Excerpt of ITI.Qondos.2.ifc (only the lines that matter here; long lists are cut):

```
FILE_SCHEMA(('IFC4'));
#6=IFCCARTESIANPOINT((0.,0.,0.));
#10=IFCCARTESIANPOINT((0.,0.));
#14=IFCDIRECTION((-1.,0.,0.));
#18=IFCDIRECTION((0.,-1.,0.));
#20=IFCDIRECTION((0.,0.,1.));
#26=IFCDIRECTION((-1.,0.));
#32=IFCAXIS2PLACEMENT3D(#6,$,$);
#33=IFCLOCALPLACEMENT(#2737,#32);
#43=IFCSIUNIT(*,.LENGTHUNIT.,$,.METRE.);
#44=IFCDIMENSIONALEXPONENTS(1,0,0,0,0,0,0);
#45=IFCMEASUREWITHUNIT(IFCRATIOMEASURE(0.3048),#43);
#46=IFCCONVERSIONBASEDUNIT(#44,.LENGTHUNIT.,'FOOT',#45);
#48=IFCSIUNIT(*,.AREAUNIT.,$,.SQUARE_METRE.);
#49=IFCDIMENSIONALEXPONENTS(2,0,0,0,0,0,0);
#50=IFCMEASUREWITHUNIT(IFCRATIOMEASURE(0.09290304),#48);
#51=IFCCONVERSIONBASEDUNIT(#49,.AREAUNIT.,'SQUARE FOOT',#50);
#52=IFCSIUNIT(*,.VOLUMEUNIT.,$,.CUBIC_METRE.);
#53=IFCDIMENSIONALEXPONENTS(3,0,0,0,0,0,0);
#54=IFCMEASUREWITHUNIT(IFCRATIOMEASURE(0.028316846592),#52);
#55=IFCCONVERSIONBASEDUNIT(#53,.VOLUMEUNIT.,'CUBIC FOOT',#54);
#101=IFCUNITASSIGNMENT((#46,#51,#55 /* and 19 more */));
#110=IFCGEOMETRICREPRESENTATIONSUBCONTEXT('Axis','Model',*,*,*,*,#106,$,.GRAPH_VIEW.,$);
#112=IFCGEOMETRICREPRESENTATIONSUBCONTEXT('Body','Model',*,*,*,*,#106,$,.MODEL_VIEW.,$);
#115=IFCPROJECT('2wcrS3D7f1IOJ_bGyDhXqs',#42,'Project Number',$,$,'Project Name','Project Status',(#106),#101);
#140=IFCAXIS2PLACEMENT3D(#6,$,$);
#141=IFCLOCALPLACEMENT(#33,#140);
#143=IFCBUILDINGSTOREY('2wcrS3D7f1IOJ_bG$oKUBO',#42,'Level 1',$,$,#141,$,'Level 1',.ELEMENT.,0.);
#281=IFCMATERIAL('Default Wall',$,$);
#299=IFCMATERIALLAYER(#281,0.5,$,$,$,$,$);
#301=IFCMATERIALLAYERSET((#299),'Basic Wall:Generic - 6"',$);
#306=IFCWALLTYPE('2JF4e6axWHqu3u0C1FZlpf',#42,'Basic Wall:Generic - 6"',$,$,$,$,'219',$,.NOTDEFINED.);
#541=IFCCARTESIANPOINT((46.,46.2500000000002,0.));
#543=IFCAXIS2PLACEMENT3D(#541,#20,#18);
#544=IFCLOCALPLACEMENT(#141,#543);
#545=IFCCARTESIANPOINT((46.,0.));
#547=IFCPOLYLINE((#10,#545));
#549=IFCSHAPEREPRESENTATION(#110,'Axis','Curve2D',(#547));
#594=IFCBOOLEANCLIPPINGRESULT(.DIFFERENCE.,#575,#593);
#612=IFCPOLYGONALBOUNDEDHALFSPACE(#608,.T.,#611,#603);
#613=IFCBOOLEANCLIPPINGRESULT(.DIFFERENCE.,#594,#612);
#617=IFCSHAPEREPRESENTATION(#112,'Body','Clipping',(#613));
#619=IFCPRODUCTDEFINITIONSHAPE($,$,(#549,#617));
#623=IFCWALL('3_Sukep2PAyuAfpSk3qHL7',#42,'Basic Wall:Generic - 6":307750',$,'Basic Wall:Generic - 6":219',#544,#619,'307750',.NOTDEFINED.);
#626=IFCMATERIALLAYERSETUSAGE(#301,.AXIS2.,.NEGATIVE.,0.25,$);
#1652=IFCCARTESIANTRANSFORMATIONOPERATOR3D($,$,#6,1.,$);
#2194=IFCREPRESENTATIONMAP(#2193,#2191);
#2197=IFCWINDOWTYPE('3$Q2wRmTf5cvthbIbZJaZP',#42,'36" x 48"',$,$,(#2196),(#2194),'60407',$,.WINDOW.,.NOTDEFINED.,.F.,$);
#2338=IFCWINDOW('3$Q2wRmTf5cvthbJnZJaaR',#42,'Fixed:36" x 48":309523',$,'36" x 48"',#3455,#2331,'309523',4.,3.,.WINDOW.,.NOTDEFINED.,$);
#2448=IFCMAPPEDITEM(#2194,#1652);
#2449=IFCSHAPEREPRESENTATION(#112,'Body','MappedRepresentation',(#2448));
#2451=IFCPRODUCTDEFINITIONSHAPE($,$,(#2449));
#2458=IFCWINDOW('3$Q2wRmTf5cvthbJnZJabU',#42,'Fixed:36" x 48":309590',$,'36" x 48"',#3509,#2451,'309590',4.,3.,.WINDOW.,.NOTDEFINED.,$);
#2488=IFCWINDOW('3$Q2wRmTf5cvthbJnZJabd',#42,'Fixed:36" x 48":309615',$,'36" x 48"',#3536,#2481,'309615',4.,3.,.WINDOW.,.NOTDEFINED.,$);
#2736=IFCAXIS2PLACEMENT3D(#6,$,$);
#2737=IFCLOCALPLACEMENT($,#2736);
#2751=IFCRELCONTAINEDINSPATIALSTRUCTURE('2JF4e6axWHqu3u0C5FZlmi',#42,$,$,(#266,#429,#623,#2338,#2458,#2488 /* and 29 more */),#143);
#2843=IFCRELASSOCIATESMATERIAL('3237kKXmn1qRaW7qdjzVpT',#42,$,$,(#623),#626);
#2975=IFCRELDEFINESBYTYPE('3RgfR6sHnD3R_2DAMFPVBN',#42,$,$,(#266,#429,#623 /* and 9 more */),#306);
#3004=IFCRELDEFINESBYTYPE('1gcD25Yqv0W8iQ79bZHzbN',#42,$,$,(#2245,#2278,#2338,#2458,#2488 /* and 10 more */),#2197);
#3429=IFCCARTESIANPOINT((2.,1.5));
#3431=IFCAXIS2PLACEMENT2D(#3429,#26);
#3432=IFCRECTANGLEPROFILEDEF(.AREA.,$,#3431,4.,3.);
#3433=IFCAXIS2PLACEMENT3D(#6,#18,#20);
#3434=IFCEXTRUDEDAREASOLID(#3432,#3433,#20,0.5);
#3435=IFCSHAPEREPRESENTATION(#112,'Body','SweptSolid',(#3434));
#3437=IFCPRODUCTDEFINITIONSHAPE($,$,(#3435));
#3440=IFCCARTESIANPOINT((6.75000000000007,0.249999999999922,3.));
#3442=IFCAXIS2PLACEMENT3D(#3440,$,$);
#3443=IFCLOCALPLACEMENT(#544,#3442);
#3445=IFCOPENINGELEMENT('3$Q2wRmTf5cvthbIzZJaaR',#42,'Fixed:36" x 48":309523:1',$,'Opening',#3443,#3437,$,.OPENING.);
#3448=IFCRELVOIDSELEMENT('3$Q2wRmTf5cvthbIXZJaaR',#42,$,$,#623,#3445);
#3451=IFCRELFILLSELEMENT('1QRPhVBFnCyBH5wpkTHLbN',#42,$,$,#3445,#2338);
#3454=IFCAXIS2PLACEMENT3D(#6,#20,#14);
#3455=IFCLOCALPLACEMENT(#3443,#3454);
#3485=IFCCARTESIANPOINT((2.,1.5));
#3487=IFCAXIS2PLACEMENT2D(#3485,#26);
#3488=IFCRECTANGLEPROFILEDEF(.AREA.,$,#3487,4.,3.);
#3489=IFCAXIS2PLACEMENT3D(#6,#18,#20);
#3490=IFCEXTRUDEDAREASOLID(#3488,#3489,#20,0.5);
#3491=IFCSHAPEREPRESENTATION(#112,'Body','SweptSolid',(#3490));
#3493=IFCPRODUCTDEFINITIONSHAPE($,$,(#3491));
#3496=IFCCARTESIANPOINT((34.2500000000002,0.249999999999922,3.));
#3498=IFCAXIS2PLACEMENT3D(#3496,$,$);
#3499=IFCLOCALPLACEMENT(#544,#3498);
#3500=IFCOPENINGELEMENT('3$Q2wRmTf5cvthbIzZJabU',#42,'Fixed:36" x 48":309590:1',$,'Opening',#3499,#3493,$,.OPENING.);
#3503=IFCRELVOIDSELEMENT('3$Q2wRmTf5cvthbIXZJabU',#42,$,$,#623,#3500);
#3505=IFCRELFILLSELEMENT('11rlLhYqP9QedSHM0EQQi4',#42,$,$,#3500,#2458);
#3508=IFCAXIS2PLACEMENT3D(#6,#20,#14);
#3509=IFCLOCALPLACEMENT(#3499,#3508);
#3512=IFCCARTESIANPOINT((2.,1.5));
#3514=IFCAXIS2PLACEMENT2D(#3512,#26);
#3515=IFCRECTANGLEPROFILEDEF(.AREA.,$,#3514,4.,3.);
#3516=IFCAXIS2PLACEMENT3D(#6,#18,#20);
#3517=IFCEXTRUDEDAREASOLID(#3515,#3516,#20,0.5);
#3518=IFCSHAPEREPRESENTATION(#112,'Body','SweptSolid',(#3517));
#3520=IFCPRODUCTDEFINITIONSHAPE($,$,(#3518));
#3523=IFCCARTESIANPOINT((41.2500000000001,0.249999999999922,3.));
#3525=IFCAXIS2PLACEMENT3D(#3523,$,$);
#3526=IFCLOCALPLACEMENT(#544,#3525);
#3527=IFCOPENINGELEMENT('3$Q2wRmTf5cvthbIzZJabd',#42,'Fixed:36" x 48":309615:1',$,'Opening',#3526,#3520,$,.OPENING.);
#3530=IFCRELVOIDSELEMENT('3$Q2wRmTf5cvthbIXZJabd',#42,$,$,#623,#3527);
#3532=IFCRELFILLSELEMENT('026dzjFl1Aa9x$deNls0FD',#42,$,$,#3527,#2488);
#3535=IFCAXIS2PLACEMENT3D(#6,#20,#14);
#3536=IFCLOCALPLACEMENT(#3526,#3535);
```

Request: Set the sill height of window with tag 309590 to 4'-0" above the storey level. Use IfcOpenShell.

```python
import numpy as np
import ifcopenshell
import ifcopenshell.api.geometry
import ifcopenshell.geom
import ifcopenshell.util.element
import ifcopenshell.util.placement
import ifcopenshell.util.shape
import ifcopenshell.util.unit

model = ifcopenshell.open("ITI.Qondos.2.ifc")
unit_scale = ifcopenshell.util.unit.calculate_unit_scale(model)

window = model.by_guid("3$Q2wRmTf5cvthbJnZJabU")
opening = window.FillsVoids[0].RelatingOpeningElement
storey = ifcopenshell.util.element.get_container(window, ifc_class="IfcBuildingStorey")
level = ifcopenshell.util.placement.get_local_placement(storey.ObjectPlacement)[2, 3]

# The opening's origin need not be at the sill, so measure its lowest point.
shape = ifcopenshell.geom.create_shape(ifcopenshell.geom.settings(), opening)
bottom = ifcopenshell.util.shape.get_shape_bottom_elevation(shape, shape.geometry) / unit_scale
dz = level + 48 * 0.0254 / unit_scale - bottom

shift = np.array([0.0, 0.0, dz])
# The window is placed relative to its opening, so it follows when the opening moves.
matrix = ifcopenshell.util.placement.get_local_placement(opening.ObjectPlacement)
matrix[:3, 3] += shift
ifcopenshell.api.geometry.edit_object_placement(
    model, product=opening, matrix=matrix, is_si=False, should_transform_children=True
)

print(f"moved by {dz * unit_scale:+.3f} m")

model.write("ITI.Qondos.2_rev.ifc")
```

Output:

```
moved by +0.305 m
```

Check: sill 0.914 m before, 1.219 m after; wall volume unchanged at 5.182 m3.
